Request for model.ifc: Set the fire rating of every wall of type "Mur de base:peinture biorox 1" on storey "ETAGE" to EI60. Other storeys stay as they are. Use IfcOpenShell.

First a look at what the model holds.

```python
import ifcopenshell
import ifcopenshell.util.element

model = ifcopenshell.open("model.ifc")
print(model.schema)
storey = next(s for s in model.by_type("IfcBuildingStorey") if s.Name == "ETAGE")
walls = [e for e in ifcopenshell.util.element.get_decomposition(storey) if e.is_a("IfcWall")]
seen = {}
for e in walls:
    element_type = ifcopenshell.util.element.get_type(e)
    key = (element_type.Name if element_type != e and element_type else None, ifcopenshell.util.element.get_pset(e, "Pset_WallCommon", "FireRating"))
    seen[key] = seen.get(key, 0) + 1
for (name, value), count in sorted(seen.items(), key=str):
    print(count, "x", name, "|", value)
```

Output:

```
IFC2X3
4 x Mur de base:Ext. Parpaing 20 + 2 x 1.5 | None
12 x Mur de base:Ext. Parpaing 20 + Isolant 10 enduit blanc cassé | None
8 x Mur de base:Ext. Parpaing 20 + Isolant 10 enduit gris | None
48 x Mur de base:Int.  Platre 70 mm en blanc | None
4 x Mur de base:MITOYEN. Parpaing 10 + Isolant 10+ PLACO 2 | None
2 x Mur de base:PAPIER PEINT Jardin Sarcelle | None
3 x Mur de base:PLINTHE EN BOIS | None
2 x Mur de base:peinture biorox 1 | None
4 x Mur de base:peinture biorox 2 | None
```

```python
import ifcopenshell
import ifcopenshell.api.pset
import ifcopenshell.util.element

model = ifcopenshell.open("model.ifc")

storey = next(s for s in model.by_type("IfcBuildingStorey") if s.Name == "ETAGE")
walls = [e for e in ifcopenshell.util.element.get_decomposition(storey) if e.is_a("IfcWall")]

count = 0
for e in walls:
    element_type = ifcopenshell.util.element.get_type(e)
    if element_type in (None, e) or element_type.Name != "Mur de base:peinture biorox 1":
        continue
    # add_pset returns the element's existing set when there is one.
    pset = ifcopenshell.api.pset.add_pset(model, product=e, name="Pset_WallCommon")
    ifcopenshell.api.pset.edit_pset(model, pset=pset, properties={"FireRating": "EI60"})
    count += 1

print(count, "walls updated")

model.write("model_rev.ifc")
```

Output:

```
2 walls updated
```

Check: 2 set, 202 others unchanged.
